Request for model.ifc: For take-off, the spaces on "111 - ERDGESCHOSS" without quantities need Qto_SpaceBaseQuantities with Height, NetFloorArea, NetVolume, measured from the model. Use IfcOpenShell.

First a look at what the model holds.

```python
import ifcopenshell
import ifcopenshell.util.element
import ifcopenshell.util.unit

model = ifcopenshell.open("model.ifc")
print(model.schema)
for unit_type in ("LENGTHUNIT", "AREAUNIT", "VOLUMEUNIT"):
    print(unit_type, ifcopenshell.util.unit.calculate_unit_scale(model, unit_type))
storey = next(s for s in model.by_type("IfcBuildingStorey") if s.Name == "111 - ERDGESCHOSS")
spaces = [e for e in ifcopenshell.util.element.get_decomposition(storey) if e.is_a("IfcSpace")]
for e in sorted(spaces, key=lambda e: e.id()):
    print(e.id(), e.is_a(), e.Name, list(ifcopenshell.util.element.get_psets(e, qtos_only=True)), sep=" | ")
```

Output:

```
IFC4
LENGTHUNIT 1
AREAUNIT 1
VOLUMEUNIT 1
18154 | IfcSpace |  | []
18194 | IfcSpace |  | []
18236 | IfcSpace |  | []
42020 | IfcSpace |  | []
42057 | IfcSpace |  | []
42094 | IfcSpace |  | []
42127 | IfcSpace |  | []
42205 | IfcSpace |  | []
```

```python
import ifcopenshell
import ifcopenshell.api.pset
import ifcopenshell.geom
import ifcopenshell.util.element
import ifcopenshell.util.shape
import ifcopenshell.util.unit

model = ifcopenshell.open("model.ifc")
unit_scale = ifcopenshell.util.unit.calculate_unit_scale(model)
area_scale = ifcopenshell.util.unit.calculate_unit_scale(model, "AREAUNIT")
volume_scale = ifcopenshell.util.unit.calculate_unit_scale(model, "VOLUMEUNIT")
settings = ifcopenshell.geom.settings()

storey = next(s for s in model.by_type("IfcBuildingStorey") if s.Name == "111 - ERDGESCHOSS")
spaces = [e for e in ifcopenshell.util.element.get_decomposition(storey) if e.is_a("IfcSpace")]

for e in sorted(spaces, key=lambda e: e.id()):
    if ifcopenshell.util.element.get_psets(e, qtos_only=True, should_inherit=False):
        continue
    # Geometry comes back in metres, in the element's own axes.
    shape = ifcopenshell.geom.create_shape(settings, e)
    values = {
        "Height": ifcopenshell.util.shape.get_z(shape.geometry) / unit_scale,
        "NetFloorArea": ifcopenshell.util.shape.get_footprint_area(shape.geometry) / area_scale,
        "NetVolume": ifcopenshell.util.shape.get_volume(shape.geometry) / volume_scale,
    }
    qto = ifcopenshell.api.pset.add_qto(model, product=e, name="Qto_SpaceBaseQuantities")
    ifcopenshell.api.pset.edit_qto(model, qto=qto, properties=values)
    print(e.id(), {k: round(v, 3) for k, v in values.items()})

model.write("model_rev.ifc")
```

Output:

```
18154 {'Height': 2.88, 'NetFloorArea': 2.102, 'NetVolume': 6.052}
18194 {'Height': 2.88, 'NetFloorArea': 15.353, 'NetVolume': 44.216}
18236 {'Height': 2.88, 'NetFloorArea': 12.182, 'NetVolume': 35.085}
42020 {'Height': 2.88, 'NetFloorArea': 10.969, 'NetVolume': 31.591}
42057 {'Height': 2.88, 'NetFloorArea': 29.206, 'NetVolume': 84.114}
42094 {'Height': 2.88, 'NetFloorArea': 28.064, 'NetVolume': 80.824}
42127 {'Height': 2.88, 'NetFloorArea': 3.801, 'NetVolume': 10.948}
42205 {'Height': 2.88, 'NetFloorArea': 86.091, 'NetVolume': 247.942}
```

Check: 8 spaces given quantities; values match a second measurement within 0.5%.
